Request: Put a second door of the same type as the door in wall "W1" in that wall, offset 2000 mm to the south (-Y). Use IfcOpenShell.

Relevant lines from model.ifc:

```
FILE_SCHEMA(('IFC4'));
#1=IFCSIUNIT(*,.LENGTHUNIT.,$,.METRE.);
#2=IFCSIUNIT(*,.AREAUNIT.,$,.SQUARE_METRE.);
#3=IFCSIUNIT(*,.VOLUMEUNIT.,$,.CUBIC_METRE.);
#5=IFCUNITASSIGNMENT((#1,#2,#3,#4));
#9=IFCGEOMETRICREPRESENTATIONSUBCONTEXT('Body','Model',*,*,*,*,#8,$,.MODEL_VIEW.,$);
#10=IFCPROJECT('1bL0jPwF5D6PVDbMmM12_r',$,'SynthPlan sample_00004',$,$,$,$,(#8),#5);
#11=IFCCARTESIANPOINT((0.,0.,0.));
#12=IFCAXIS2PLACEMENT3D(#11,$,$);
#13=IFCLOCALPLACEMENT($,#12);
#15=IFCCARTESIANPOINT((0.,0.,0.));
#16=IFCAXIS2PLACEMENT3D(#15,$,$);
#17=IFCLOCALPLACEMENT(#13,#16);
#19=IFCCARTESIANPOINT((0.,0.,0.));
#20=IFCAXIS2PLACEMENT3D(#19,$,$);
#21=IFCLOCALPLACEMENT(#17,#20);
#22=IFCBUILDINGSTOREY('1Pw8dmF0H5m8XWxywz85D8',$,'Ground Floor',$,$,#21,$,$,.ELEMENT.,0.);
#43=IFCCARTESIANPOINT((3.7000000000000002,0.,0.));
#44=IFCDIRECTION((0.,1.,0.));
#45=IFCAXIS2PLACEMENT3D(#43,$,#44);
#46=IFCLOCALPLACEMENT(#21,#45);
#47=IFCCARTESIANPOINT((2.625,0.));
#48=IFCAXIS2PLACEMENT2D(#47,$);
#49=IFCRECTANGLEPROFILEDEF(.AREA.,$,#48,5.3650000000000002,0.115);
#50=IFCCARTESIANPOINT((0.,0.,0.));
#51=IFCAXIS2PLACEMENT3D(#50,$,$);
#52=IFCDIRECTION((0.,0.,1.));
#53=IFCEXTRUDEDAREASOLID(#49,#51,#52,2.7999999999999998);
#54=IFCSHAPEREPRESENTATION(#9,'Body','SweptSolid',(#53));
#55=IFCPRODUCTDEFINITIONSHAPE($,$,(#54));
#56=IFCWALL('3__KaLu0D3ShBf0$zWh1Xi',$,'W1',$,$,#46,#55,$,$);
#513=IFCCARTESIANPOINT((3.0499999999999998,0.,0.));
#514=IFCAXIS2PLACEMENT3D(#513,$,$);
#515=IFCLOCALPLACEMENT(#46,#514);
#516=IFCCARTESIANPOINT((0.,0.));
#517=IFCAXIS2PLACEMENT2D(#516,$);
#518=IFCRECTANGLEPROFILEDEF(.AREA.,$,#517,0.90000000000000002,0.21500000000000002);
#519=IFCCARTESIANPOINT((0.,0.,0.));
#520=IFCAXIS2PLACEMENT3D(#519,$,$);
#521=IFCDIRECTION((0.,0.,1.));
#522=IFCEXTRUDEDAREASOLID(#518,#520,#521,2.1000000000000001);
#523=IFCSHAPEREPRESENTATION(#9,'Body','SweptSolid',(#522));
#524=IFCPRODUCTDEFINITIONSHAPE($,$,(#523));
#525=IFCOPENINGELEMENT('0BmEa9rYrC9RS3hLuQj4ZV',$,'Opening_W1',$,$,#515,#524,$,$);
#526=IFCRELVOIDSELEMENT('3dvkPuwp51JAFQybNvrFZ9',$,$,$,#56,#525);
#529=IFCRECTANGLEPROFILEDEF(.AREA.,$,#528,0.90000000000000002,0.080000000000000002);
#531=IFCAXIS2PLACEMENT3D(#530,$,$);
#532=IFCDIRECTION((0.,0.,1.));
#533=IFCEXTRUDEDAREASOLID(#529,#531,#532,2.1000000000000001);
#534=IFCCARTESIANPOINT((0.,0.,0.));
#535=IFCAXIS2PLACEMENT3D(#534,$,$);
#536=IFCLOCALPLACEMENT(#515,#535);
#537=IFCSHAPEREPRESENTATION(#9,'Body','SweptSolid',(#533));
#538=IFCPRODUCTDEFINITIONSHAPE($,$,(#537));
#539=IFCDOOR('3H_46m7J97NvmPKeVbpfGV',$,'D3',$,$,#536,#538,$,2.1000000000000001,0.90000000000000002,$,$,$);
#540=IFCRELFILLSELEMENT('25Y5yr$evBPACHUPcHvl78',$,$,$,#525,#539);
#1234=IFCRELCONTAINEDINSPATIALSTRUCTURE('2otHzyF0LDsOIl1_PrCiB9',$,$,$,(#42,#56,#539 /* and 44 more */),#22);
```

```python
import ifcopenshell
import ifcopenshell.api.feature
import ifcopenshell.api.geometry
import ifcopenshell.api.root
import ifcopenshell.geom
import ifcopenshell.util.element
import ifcopenshell.util.placement
import ifcopenshell.util.shape
import ifcopenshell.util.unit

model = ifcopenshell.open("model.ifc")
unit_scale = ifcopenshell.util.unit.calculate_unit_scale(model)
settings = ifcopenshell.geom.settings()


def volume(element):
    """Net volume in cubic metres, openings subtracted."""
    shape = ifcopenshell.geom.create_shape(settings, element)
    return ifcopenshell.util.shape.get_volume(shape.geometry)


door = model.by_guid("3H_46m7J97NvmPKeVbpfGV")
opening = door.FillsVoids[0].RelatingOpeningElement
wall = opening.VoidsElements[0].RelatingBuildingElement
before = volume(wall)
shift = ifcopenshell.util.placement.get_local_placement(wall.ObjectPlacement)[:3, 0] * -2 / unit_scale

# copy_class copies the void relationship, type, container and properties, but no geometry.
new_opening = ifcopenshell.api.root.copy_class(model, product=opening)
new_opening.Representation = ifcopenshell.util.element.copy_deep(
    model, opening.Representation, exclude=["IfcGeometricRepresentationContext", "IfcRepresentationMap"]
)
new_door = ifcopenshell.api.root.copy_class(model, product=door)
new_door.Representation = ifcopenshell.util.element.copy_deep(
    model, door.Representation, exclude=["IfcGeometricRepresentationContext", "IfcRepresentationMap"]
)
ifcopenshell.api.feature.add_filling(model, opening=new_opening, element=new_door)

for old, new in ((opening, new_opening), (door, new_door)):
    matrix = ifcopenshell.util.placement.get_local_placement(old.ObjectPlacement)
    matrix[:3, 3] += shift
    ifcopenshell.api.geometry.edit_object_placement(model, product=new, matrix=matrix, is_si=False)

after = volume(wall)

print(f"wall volume {before:.3f} -> {after:.3f} m3")

model.write("model_edited.ifc")
```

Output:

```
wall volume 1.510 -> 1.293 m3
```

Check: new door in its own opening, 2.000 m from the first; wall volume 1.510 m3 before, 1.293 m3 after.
